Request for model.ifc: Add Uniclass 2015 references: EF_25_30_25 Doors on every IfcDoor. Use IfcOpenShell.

First a look at what the model holds.

```python
import ifcopenshell

model = ifcopenshell.open("model.ifc")
print(model.schema)
print("classifications:", [c.Name for c in model.by_type("IfcClassification")])
for ifc_class in ("IfcDoor", "IfcRoof", "IfcStair", "IfcWall", "IfcWindow"):
    print(ifc_class, len(model.by_type(ifc_class)))
```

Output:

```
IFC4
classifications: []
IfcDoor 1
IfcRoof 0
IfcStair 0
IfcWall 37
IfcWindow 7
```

```python
import ifcopenshell
import ifcopenshell.api.classification

model = ifcopenshell.open("model.ifc")

system = ifcopenshell.api.classification.add_classification(model, classification="Uniclass 2015")

codes = {
    "IfcDoor": ("EF_25_30_25", "Doors"),
}
for ifc_class, (code, name) in codes.items():
    products = model.by_type(ifc_class)
    ifcopenshell.api.classification.add_reference(
        model, products=products, classification=system, identification=code, name=name
    )
    print(code, len(products))

model.write("model_v2.ifc")
```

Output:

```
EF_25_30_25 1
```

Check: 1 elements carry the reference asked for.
